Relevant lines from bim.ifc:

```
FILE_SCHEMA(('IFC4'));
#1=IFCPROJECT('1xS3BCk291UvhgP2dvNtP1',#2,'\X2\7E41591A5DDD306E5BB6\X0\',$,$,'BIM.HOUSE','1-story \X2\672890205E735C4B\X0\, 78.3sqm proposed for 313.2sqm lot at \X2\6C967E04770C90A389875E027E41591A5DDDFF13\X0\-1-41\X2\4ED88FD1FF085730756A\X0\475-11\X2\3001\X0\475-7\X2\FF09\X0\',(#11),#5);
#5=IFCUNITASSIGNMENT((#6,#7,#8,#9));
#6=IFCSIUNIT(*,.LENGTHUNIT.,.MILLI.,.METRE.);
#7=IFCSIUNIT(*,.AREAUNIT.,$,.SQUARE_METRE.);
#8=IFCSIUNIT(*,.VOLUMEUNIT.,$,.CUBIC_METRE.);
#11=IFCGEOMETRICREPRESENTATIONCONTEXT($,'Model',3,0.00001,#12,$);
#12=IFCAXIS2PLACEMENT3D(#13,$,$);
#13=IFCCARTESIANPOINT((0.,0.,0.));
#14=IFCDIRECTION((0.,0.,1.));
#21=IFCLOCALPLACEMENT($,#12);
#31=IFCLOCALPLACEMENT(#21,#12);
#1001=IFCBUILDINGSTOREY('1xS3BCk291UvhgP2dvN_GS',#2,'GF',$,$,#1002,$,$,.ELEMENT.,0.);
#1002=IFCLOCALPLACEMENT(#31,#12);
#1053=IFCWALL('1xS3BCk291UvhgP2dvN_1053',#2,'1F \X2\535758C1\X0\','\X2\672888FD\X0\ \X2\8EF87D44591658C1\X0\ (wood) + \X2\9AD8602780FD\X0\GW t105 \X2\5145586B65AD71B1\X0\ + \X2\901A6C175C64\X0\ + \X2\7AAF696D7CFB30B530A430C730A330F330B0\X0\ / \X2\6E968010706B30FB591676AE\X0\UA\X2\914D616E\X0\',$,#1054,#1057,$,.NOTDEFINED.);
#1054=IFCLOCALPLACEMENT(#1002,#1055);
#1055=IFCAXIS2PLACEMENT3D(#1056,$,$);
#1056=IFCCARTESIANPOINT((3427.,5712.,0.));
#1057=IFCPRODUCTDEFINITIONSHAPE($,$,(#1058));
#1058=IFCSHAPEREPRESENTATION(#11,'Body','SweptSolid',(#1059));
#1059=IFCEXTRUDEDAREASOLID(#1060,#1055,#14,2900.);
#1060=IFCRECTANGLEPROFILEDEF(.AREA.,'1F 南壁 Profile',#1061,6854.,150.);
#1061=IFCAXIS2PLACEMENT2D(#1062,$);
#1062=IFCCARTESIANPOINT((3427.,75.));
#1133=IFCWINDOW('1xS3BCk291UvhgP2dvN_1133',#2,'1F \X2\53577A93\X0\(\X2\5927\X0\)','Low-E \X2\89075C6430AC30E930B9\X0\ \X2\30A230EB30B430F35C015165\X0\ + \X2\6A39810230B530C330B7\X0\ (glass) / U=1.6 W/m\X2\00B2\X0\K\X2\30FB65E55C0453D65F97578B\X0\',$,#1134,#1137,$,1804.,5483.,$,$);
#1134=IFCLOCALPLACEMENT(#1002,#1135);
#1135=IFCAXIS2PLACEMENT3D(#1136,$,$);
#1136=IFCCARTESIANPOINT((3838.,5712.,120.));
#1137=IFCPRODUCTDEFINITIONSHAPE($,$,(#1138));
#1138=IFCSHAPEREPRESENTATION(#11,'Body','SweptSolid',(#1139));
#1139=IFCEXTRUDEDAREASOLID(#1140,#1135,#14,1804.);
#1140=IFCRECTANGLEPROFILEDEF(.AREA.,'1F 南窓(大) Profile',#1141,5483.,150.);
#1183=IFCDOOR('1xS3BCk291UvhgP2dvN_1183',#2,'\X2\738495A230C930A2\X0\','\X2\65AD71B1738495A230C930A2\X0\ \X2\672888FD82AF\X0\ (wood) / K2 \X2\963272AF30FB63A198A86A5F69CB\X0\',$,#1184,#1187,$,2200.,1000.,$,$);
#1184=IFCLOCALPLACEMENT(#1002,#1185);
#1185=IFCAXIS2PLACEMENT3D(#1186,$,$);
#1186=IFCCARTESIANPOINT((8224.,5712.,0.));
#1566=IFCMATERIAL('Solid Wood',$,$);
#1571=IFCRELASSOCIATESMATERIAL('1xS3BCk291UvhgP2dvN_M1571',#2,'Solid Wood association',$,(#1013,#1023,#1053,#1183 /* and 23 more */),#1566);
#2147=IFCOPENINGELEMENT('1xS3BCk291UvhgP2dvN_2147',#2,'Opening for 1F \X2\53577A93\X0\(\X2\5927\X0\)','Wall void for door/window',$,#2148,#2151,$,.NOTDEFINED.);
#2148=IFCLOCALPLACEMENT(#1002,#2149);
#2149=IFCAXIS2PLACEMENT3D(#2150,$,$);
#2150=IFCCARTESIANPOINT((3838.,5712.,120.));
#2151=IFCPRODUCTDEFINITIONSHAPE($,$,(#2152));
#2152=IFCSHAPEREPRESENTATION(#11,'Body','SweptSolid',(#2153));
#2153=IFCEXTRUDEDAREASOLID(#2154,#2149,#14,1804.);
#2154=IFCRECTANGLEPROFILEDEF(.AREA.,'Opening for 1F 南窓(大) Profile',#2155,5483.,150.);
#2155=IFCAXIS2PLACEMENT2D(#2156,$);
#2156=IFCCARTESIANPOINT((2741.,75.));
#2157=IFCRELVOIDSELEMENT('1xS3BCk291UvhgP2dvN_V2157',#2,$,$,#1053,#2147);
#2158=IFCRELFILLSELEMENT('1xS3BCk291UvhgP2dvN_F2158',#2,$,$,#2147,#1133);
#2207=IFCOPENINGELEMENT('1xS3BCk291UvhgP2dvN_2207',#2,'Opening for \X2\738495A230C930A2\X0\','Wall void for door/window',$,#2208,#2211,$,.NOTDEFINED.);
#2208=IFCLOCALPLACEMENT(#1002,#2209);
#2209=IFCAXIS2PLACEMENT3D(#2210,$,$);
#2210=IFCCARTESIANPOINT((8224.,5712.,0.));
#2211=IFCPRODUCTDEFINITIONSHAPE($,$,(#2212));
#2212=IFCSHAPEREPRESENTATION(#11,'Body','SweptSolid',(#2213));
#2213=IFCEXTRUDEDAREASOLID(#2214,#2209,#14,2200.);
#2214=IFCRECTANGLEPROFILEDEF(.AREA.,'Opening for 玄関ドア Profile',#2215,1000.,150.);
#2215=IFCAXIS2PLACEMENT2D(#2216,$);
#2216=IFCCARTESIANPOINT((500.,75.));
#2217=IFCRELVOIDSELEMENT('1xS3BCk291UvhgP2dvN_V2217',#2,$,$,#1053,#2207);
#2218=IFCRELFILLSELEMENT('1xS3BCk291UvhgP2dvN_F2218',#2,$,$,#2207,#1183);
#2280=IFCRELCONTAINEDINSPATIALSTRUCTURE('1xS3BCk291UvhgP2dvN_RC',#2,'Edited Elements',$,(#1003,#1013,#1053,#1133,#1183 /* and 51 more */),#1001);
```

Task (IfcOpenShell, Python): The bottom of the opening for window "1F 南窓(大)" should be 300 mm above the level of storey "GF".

```python
import numpy as np
import ifcopenshell
import ifcopenshell.api.geometry
import ifcopenshell.geom
import ifcopenshell.util.element
import ifcopenshell.util.placement
import ifcopenshell.util.shape
import ifcopenshell.util.unit

model = ifcopenshell.open("bim.ifc")
unit_scale = ifcopenshell.util.unit.calculate_unit_scale(model)

window = model.by_id(1133)
opening = window.FillsVoids[0].RelatingOpeningElement
storey = ifcopenshell.util.element.get_container(window, ifc_class="IfcBuildingStorey")
level = ifcopenshell.util.placement.get_local_placement(storey.ObjectPlacement)[2, 3]

# The opening's origin need not be at the sill, so measure its lowest point.
shape = ifcopenshell.geom.create_shape(ifcopenshell.geom.settings(), opening)
bottom = ifcopenshell.util.shape.get_shape_bottom_elevation(shape, shape.geometry) / unit_scale
dz = level + 0.3 / unit_scale - bottom

shift = np.array([0.0, 0.0, dz])
# The window is not placed relative to its opening, so move both.
for product in (opening, window):
    matrix = ifcopenshell.util.placement.get_local_placement(product.ObjectPlacement)
    matrix[:3, 3] += shift
    ifcopenshell.api.geometry.edit_object_placement(model, product=product, matrix=matrix, is_si=False)

print(f"moved by {dz * unit_scale:+.3f} m")

model.write("bim_rev.ifc")
```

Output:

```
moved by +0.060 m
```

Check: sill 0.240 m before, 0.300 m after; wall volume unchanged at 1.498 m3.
